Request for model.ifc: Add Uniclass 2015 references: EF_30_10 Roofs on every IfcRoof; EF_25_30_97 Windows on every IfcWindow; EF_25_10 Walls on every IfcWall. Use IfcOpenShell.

First a look at what the model holds.

```python
import ifcopenshell

model = ifcopenshell.open("model.ifc")
print(model.schema)
print("classifications:", [c.Name for c in model.by_type("IfcClassification")])
for ifc_class in ("IfcDoor", "IfcRoof", "IfcStair", "IfcWall", "IfcWindow"):
    print(ifc_class, len(model.by_type(ifc_class)))
```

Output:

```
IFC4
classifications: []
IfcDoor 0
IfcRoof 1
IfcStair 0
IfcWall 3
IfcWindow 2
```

```python
import ifcopenshell
import ifcopenshell.api.classification

model = ifcopenshell.open("model.ifc")

system = ifcopenshell.api.classification.add_classification(model, classification="Uniclass 2015")

codes = {
    "IfcRoof": ("EF_30_10", "Roofs"),
    "IfcWindow": ("EF_25_30_97", "Windows"),
    "IfcWall": ("EF_25_10", "Walls"),
}
for ifc_class, (code, name) in codes.items():
    products = model.by_type(ifc_class)
    ifcopenshell.api.classification.add_reference(
        model, products=products, classification=system, identification=code, name=name
    )
    print(code, len(products))

model.write("model_v2.ifc")
```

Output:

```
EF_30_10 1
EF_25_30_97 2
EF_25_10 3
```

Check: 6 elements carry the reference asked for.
